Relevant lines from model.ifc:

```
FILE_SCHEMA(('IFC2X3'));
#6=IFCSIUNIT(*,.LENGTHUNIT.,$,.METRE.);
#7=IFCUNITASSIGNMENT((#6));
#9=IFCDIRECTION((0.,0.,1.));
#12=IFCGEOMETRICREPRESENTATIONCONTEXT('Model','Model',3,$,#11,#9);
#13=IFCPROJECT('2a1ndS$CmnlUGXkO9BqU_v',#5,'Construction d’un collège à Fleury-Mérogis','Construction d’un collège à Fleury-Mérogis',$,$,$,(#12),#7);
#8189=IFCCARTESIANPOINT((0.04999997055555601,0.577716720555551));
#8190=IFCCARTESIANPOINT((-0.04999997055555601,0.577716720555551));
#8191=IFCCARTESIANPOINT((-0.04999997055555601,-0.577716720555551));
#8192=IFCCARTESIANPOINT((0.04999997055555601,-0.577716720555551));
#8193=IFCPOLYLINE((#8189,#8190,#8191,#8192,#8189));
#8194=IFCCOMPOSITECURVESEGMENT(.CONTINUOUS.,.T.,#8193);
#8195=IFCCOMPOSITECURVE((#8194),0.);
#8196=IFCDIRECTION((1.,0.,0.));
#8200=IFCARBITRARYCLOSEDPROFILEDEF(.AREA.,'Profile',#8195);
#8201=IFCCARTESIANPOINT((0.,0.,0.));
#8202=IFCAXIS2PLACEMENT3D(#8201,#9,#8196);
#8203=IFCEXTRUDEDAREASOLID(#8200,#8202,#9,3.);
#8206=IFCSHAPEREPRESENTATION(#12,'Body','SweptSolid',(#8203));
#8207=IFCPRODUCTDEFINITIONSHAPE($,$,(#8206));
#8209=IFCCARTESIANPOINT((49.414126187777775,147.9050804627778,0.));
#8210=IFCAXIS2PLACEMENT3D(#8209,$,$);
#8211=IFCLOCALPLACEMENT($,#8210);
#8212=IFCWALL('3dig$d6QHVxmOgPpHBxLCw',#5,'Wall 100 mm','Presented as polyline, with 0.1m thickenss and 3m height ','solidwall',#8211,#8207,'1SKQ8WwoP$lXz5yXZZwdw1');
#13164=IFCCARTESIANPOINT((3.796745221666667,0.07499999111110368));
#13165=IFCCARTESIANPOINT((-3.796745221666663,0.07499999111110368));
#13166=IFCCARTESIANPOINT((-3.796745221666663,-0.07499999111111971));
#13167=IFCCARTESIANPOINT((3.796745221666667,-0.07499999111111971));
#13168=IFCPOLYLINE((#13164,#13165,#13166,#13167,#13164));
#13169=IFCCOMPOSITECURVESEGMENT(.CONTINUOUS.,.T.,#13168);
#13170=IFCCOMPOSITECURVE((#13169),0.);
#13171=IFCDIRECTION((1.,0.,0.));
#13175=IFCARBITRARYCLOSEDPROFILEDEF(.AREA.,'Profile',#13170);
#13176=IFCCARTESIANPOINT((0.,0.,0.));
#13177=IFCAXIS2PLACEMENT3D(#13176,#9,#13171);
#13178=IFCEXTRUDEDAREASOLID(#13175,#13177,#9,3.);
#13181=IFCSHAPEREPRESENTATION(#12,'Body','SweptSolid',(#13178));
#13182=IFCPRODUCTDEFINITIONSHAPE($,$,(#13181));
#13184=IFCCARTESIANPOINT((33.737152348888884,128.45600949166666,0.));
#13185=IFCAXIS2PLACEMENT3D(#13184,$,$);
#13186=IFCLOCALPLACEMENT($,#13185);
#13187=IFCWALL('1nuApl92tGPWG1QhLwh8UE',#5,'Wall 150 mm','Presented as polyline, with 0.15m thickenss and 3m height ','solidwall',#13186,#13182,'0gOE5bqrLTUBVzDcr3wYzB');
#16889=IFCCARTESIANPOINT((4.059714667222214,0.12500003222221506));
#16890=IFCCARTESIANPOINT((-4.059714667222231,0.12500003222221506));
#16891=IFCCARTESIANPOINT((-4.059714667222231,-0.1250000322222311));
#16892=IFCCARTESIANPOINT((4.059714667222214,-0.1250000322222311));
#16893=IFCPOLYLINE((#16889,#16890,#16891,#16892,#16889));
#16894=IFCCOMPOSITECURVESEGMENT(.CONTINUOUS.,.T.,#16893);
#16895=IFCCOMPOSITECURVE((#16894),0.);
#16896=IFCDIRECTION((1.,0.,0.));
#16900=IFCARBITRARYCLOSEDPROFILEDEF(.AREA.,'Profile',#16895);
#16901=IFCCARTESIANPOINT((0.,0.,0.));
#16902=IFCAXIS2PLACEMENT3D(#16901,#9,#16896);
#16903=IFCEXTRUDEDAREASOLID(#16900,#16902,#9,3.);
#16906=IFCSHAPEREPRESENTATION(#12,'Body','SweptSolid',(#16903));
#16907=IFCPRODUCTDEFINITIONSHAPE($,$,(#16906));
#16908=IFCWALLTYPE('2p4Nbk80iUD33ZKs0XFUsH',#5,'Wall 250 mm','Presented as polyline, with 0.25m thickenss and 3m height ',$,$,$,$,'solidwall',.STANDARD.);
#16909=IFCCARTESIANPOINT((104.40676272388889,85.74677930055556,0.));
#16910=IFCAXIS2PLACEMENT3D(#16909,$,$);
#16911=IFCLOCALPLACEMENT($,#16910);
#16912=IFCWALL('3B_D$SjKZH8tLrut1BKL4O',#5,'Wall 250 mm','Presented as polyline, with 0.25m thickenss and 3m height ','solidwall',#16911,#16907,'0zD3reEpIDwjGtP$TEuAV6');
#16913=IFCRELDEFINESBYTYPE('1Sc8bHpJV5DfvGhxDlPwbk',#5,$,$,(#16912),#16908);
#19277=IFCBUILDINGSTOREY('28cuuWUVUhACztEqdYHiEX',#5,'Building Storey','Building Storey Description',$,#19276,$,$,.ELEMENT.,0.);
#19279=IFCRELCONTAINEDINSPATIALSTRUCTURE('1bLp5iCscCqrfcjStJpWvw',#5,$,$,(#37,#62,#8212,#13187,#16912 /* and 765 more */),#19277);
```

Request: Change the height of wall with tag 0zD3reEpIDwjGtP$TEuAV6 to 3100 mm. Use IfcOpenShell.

```python
import ifcopenshell
import ifcopenshell.geom
import ifcopenshell.util.shape
import ifcopenshell.util.unit

model = ifcopenshell.open("model.ifc")
unit_scale = ifcopenshell.util.unit.calculate_unit_scale(model)
settings = ifcopenshell.geom.settings()


def volume(element):
    """Net volume in cubic metres, openings subtracted."""
    shape = ifcopenshell.geom.create_shape(settings, element)
    return ifcopenshell.util.shape.get_volume(shape.geometry)


wall = model.by_guid("3B_D$SjKZH8tLrut1BKL4O")
before = volume(wall)

body = next(r for r in wall.Representation.Representations if r.RepresentationIdentifier == "Body")
solid = body.Items[0]
old_height = solid.Depth
solid.Depth = 3.1 / unit_scale
after = volume(wall)

print(f"height {old_height:g} -> {solid.Depth:g}, volume {before:.3f} -> {after:.3f} m3")

model.write("model_edited.ifc")
```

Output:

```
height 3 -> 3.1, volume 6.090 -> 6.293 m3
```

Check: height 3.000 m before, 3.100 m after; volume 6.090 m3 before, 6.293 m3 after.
